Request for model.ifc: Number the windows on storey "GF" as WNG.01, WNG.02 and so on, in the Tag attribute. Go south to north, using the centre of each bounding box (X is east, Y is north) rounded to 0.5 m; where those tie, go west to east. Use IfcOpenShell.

First a look at what the model holds.

```python
import ifcopenshell
import ifcopenshell.util.element
import ifcopenshell.util.placement

model = ifcopenshell.open("model.ifc")
print(model.schema)
storey = next(s for s in model.by_type("IfcBuildingStorey") if s.Name == "GF")
windows = [e for e in ifcopenshell.util.element.get_decomposition(storey) if e.is_a("IfcWindow")]
for e in sorted(windows, key=lambda e: e.id()):
    origin = ifcopenshell.util.placement.get_local_placement(e.ObjectPlacement)[:3, 3]
    print(e.id(), e.Tag, e.Name, origin.round(2) + 0.0, sep=" | ")
```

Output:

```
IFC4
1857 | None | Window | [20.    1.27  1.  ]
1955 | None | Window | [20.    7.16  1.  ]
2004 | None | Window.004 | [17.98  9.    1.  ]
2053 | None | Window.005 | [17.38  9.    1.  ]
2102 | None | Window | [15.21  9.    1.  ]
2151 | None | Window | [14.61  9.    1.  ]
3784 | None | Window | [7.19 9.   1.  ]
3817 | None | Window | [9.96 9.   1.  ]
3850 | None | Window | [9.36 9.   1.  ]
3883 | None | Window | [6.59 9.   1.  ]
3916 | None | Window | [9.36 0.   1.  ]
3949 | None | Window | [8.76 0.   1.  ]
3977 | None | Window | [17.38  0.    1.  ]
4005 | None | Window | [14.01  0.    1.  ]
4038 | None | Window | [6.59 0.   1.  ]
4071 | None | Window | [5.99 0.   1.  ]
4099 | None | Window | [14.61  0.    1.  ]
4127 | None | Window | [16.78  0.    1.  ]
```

```python
import ifcopenshell
import ifcopenshell.geom
import ifcopenshell.util.element
import ifcopenshell.util.shape

model = ifcopenshell.open("model.ifc")
settings = ifcopenshell.geom.settings()
settings.set("use-world-coords", True)


def centre(element):
    shape = ifcopenshell.geom.create_shape(settings, element)
    return ifcopenshell.util.shape.get_bbox_centroid(shape.geometry)


storey = next(s for s in model.by_type("IfcBuildingStorey") if s.Name == "GF")
windows = [e for e in ifcopenshell.util.element.get_decomposition(storey) if e.is_a("IfcWindow")]

# Insertion points can sit at a corner or the storey origin, so sort by the geometry (in metres).
centres = {e: centre(e) for e in windows}
windows.sort(key=lambda e: (round(centres[e][1] / 0.5), centres[e][0]))

for i, e in enumerate(windows, start=1):
    number = f"WNG.{i:02d}"
    e.Tag = number
    print(e.id(), number)

model.write("model_updated.ifc")
```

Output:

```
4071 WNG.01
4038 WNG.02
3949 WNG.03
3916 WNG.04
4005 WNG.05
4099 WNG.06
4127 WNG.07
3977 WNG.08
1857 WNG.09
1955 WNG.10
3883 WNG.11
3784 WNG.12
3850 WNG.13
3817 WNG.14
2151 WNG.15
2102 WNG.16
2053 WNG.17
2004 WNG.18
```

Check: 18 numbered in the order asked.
